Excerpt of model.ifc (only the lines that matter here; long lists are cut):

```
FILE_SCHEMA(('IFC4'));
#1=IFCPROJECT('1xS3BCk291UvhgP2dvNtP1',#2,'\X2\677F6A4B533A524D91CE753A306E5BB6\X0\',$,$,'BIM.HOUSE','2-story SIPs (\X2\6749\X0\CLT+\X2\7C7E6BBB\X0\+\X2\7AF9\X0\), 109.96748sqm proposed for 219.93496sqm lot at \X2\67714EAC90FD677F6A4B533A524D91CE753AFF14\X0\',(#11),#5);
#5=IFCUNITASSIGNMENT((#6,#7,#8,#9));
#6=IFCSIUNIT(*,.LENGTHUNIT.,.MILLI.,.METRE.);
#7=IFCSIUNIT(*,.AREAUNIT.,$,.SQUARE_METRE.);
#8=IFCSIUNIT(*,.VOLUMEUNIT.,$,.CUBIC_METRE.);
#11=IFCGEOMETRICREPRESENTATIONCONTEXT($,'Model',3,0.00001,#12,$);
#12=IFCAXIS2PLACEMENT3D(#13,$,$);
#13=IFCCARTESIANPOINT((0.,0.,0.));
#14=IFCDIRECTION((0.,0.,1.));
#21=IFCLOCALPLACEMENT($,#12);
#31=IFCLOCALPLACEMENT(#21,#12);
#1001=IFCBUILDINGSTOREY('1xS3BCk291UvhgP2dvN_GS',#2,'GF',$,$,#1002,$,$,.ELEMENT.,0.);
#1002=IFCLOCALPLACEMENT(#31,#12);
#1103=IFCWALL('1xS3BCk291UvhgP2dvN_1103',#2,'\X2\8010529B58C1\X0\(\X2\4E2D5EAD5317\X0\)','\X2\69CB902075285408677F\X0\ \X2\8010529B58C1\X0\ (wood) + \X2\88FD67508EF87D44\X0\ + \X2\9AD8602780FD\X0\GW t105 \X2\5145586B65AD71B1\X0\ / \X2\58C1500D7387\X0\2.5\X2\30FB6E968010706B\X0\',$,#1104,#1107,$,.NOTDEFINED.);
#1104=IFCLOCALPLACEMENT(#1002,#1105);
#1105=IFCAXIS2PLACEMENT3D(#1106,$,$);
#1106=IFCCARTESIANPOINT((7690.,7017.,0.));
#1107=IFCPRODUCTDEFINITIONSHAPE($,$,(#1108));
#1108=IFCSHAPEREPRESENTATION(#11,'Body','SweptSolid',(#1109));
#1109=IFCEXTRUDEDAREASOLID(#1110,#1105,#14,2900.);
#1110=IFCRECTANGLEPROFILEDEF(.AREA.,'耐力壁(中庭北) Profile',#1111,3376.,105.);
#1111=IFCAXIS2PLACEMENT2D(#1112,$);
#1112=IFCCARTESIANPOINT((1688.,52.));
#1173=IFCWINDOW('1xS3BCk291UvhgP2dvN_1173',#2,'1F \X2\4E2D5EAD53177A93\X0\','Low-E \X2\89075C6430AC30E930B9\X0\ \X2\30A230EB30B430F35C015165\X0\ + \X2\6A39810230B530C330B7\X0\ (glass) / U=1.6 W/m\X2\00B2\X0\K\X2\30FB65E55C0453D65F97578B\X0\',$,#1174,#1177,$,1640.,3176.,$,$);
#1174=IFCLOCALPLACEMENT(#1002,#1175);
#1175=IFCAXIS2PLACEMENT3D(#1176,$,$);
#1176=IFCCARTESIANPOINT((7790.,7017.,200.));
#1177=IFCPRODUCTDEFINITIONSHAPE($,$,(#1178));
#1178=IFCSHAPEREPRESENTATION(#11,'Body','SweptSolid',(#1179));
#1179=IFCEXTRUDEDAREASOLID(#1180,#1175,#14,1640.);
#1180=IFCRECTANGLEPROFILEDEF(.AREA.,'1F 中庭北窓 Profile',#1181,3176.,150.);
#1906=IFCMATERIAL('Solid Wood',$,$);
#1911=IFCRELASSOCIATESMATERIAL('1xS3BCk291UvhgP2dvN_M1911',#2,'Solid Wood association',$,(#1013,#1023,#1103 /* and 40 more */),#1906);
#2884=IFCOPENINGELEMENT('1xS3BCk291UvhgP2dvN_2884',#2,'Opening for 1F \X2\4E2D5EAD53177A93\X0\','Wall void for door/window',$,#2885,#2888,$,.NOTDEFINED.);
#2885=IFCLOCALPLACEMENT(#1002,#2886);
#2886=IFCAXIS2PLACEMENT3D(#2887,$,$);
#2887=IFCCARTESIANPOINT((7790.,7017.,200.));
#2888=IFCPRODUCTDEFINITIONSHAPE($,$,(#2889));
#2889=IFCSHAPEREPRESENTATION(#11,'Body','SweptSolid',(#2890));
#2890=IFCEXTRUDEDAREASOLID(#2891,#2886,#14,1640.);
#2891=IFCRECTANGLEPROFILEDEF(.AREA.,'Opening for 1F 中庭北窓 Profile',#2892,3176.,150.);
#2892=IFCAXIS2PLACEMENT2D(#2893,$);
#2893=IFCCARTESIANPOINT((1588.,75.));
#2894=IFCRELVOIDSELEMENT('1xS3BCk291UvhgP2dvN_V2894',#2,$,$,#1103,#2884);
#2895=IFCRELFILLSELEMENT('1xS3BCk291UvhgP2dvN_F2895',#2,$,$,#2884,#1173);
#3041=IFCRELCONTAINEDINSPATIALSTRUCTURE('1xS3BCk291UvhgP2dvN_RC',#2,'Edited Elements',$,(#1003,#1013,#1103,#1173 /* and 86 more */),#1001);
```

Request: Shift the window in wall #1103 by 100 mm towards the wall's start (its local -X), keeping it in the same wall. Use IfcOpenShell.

```python
import ifcopenshell
import ifcopenshell.api.geometry
import ifcopenshell.util.placement
import ifcopenshell.util.unit

model = ifcopenshell.open("model.ifc")
unit_scale = ifcopenshell.util.unit.calculate_unit_scale(model)

window = model.by_guid("1xS3BCk291UvhgP2dvN_1173")
opening = window.FillsVoids[0].RelatingOpeningElement
wall = opening.VoidsElements[0].RelatingBuildingElement

wall_matrix = ifcopenshell.util.placement.get_local_placement(wall.ObjectPlacement)
shift = wall_matrix[:3, 0] * -0.1 / unit_scale
before = ifcopenshell.util.placement.get_local_placement(window.ObjectPlacement)[:3, 3].copy()

# The window is not placed relative to its opening, so move both.
for product in (opening, window):
    matrix = ifcopenshell.util.placement.get_local_placement(product.ObjectPlacement)
    matrix[:3, 3] += shift
    ifcopenshell.api.geometry.edit_object_placement(model, product=product, matrix=matrix, is_si=False)

after = ifcopenshell.util.placement.get_local_placement(window.ObjectPlacement)[:3, 3]
print("window moved by", (after - before).round(3) + 0.0)

model.write("model_edited.ifc")
```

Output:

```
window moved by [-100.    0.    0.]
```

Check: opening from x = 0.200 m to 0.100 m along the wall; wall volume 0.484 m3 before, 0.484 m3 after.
